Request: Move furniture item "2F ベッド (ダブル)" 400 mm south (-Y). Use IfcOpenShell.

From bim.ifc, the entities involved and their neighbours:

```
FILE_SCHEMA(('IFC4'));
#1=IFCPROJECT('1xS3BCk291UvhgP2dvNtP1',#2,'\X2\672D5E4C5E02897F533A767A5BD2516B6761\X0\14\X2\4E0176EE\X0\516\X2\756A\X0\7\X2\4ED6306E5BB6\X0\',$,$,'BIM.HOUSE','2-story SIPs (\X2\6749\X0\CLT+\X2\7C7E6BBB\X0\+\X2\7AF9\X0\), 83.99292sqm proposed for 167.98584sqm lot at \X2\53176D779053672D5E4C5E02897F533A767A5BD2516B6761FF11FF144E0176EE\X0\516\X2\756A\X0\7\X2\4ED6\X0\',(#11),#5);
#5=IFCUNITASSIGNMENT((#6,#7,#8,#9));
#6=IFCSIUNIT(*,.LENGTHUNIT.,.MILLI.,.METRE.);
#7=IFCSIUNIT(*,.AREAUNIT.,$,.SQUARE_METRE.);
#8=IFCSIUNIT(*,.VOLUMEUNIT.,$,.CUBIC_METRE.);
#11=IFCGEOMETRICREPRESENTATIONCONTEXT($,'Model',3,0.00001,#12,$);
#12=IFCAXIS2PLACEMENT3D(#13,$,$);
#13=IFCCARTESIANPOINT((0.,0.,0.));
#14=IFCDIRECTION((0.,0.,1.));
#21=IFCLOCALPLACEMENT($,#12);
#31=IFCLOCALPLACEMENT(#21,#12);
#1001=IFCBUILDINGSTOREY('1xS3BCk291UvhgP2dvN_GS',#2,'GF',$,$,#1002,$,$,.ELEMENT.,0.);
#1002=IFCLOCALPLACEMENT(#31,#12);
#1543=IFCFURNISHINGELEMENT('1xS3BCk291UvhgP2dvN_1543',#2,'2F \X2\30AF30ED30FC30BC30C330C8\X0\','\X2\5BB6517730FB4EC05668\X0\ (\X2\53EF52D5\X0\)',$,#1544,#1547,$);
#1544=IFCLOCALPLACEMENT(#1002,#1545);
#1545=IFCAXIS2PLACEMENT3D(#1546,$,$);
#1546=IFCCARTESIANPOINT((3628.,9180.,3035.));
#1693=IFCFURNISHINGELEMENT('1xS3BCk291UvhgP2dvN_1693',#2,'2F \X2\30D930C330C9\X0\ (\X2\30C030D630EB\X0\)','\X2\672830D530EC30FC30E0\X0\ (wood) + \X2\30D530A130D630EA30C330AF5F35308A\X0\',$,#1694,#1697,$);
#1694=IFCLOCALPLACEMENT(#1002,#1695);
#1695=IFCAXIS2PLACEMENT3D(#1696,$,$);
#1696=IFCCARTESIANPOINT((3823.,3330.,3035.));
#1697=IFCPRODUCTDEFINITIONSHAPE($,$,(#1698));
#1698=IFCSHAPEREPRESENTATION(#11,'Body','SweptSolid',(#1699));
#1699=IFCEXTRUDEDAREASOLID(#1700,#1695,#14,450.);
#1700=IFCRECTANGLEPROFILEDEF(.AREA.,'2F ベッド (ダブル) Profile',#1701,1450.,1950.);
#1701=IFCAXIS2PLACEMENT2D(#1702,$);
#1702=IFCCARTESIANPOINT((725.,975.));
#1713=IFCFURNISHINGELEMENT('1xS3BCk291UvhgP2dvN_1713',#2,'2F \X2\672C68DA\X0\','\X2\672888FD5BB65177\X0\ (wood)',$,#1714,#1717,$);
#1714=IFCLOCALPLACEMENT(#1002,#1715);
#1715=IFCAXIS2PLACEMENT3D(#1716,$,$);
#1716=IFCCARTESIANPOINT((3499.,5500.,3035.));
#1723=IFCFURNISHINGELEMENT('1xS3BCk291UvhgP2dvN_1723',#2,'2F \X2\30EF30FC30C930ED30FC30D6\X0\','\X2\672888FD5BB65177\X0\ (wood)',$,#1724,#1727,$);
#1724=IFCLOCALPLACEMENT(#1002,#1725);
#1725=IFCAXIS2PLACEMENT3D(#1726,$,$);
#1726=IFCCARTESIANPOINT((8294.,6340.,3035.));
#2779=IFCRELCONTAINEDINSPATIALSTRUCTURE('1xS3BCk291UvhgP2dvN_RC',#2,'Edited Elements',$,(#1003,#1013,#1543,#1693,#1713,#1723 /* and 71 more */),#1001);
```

```python
import ifcopenshell
import ifcopenshell.api.geometry
import ifcopenshell.util.placement

model = ifcopenshell.open("bim.ifc")

item = model.by_guid("1xS3BCk291UvhgP2dvN_1693")
matrix = ifcopenshell.util.placement.get_local_placement(item.ObjectPlacement)
matrix[1, 3] -= 400.0
ifcopenshell.api.geometry.edit_object_placement(model, product=item, matrix=matrix, is_si=False)

print(ifcopenshell.util.placement.get_local_placement(item.ObjectPlacement).round(3) + 0.0)

model.write("bim_rev.ifc")
```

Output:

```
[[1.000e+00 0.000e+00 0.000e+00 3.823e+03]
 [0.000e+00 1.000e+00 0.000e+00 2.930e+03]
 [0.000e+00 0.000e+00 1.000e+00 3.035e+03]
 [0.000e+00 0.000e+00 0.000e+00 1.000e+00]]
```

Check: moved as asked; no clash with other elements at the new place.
